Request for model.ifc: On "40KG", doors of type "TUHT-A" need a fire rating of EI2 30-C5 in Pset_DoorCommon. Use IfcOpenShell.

First a look at what the model holds.

```python
import ifcopenshell
import ifcopenshell.util.element

model = ifcopenshell.open("model.ifc")
print(model.schema)
storey = next(s for s in model.by_type("IfcBuildingStorey") if s.Name == "40KG")
doors = [e for e in ifcopenshell.util.element.get_decomposition(storey) if e.is_a("IfcDoor")]
seen = {}
for e in doors:
    element_type = ifcopenshell.util.element.get_type(e)
    key = (element_type.Name if element_type != e and element_type else None, ifcopenshell.util.element.get_pset(e, "Pset_DoorCommon", "FireRating"))
    seen[key] = seen.get(key, 0) + 1
for (name, value), count in sorted(seen.items(), key=str):
    print(count, "x", name, "|", value)
```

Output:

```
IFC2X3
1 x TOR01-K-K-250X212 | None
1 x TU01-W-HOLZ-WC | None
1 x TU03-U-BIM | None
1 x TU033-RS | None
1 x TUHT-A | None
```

```python
import ifcopenshell
import ifcopenshell.api.pset
import ifcopenshell.util.element

model = ifcopenshell.open("model.ifc")

storey = next(s for s in model.by_type("IfcBuildingStorey") if s.Name == "40KG")
doors = [e for e in ifcopenshell.util.element.get_decomposition(storey) if e.is_a("IfcDoor")]

count = 0
for e in doors:
    element_type = ifcopenshell.util.element.get_type(e)
    if element_type in (None, e) or element_type.Name != "TUHT-A":
        continue
    # add_pset returns the element's existing set when there is one.
    pset = ifcopenshell.api.pset.add_pset(model, product=e, name="Pset_DoorCommon")
    ifcopenshell.api.pset.edit_pset(model, pset=pset, properties={"FireRating": "EI2 30-C5"})
    count += 1

print(count, "doors updated")

model.write("model_v2.ifc")
```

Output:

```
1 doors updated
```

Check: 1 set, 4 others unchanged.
